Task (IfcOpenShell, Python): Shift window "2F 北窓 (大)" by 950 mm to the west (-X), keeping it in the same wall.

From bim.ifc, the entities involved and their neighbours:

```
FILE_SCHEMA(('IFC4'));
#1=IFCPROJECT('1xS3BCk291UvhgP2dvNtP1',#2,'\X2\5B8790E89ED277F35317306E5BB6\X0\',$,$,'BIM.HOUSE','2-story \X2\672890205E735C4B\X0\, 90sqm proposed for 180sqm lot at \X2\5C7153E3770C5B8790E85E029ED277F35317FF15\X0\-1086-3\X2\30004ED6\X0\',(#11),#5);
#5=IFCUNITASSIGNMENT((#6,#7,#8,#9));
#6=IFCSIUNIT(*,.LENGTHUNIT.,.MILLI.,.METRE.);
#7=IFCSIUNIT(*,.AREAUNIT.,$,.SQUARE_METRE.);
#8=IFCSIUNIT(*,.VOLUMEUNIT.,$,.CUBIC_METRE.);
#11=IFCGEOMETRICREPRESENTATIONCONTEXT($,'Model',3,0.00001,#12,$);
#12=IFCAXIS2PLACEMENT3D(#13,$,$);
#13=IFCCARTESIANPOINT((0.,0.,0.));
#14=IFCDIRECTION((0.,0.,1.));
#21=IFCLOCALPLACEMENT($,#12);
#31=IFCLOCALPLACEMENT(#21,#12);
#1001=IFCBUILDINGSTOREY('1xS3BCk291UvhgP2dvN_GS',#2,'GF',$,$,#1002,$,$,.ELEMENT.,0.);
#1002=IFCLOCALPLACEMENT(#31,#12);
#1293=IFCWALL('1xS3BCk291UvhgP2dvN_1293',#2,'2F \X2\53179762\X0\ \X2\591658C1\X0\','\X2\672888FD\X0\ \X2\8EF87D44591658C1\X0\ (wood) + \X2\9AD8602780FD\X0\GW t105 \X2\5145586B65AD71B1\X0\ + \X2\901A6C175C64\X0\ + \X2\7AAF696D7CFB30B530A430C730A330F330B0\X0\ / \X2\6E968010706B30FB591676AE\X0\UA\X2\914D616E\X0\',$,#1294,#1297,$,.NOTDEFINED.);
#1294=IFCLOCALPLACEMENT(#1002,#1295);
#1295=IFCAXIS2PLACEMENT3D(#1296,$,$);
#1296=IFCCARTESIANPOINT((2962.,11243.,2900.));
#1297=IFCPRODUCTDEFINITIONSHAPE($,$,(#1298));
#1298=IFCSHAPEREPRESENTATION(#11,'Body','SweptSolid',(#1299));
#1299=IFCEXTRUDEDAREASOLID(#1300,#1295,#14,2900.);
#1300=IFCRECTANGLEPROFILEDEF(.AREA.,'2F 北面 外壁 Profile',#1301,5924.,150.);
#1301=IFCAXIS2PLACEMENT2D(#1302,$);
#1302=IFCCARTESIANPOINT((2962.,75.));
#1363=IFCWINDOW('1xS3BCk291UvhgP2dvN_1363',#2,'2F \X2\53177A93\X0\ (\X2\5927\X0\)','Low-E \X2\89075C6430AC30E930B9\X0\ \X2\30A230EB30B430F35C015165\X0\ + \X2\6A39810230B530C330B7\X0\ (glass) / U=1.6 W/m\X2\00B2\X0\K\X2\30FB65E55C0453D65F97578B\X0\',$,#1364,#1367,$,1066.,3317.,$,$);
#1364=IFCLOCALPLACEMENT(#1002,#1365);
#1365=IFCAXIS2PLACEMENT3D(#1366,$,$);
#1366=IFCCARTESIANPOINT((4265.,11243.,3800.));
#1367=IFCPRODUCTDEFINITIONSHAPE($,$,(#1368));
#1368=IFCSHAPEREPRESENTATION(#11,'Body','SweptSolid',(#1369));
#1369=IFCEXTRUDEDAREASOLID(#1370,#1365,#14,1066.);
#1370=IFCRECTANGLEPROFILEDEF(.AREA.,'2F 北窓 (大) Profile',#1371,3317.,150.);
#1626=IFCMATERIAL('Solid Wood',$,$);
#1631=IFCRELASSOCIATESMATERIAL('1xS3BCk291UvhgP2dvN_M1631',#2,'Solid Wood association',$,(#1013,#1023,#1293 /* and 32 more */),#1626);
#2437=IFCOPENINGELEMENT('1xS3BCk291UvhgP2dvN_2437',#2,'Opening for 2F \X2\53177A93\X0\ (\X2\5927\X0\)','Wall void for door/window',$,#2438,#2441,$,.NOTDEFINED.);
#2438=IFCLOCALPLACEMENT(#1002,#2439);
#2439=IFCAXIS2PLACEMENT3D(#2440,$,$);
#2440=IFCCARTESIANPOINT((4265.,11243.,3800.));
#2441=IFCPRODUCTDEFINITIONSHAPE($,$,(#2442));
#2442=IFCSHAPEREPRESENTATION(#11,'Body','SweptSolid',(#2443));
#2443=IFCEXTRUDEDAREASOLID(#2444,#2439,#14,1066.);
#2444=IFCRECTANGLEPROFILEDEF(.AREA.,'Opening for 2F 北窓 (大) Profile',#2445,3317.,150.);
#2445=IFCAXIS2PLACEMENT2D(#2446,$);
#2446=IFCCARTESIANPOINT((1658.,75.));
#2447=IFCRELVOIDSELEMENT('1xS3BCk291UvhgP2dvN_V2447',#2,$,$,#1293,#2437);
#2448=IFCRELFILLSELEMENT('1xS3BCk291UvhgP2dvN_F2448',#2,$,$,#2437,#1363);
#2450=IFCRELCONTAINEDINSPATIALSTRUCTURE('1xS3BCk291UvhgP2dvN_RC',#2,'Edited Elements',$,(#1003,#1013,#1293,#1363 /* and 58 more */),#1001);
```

```python
import ifcopenshell
import ifcopenshell.api.geometry
import ifcopenshell.util.placement
import ifcopenshell.util.unit

model = ifcopenshell.open("bim.ifc")
unit_scale = ifcopenshell.util.unit.calculate_unit_scale(model)

window = model.by_guid("1xS3BCk291UvhgP2dvN_1363")
opening = window.FillsVoids[0].RelatingOpeningElement
wall = opening.VoidsElements[0].RelatingBuildingElement

wall_matrix = ifcopenshell.util.placement.get_local_placement(wall.ObjectPlacement)
shift = wall_matrix[:3, 0] * -0.95 / unit_scale
before = ifcopenshell.util.placement.get_local_placement(window.ObjectPlacement)[:3, 3].copy()

# The window is not placed relative to its opening, so move both.
for product in (opening, window):
    matrix = ifcopenshell.util.placement.get_local_placement(product.ObjectPlacement)
    matrix[:3, 3] += shift
    ifcopenshell.api.geometry.edit_object_placement(model, product=product, matrix=matrix, is_si=False)

after = ifcopenshell.util.placement.get_local_placement(window.ObjectPlacement)[:3, 3]
print("window moved by", (after - before).round(3) + 0.0)

model.write("bim_updated.ifc")
```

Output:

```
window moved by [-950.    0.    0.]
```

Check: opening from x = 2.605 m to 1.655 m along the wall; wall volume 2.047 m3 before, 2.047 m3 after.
